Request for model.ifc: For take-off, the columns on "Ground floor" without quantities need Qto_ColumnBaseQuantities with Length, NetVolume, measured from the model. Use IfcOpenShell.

First a look at what the model holds.

```python
import ifcopenshell
import ifcopenshell.util.element
import ifcopenshell.util.unit

model = ifcopenshell.open("model.ifc")
print(model.schema)
for unit_type in ("LENGTHUNIT", "AREAUNIT", "VOLUMEUNIT"):
    print(unit_type, ifcopenshell.util.unit.calculate_unit_scale(model, unit_type))
storey = next(s for s in model.by_type("IfcBuildingStorey") if s.Name == "Ground floor")
columns = [e for e in ifcopenshell.util.element.get_decomposition(storey) if e.is_a("IfcColumn")]
for e in sorted(columns, key=lambda e: e.id()):
    print(e.id(), e.is_a(), e.Name, list(ifcopenshell.util.element.get_psets(e, qtos_only=True)), sep=" | ")
```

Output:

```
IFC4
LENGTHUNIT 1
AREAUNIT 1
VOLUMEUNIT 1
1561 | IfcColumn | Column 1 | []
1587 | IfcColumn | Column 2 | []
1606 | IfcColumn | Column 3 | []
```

```python
import ifcopenshell
import ifcopenshell.api.pset
import ifcopenshell.geom
import ifcopenshell.util.element
import ifcopenshell.util.shape
import ifcopenshell.util.unit

model = ifcopenshell.open("model.ifc")
unit_scale = ifcopenshell.util.unit.calculate_unit_scale(model)
volume_scale = ifcopenshell.util.unit.calculate_unit_scale(model, "VOLUMEUNIT")
settings = ifcopenshell.geom.settings()

storey = next(s for s in model.by_type("IfcBuildingStorey") if s.Name == "Ground floor")
columns = [e for e in ifcopenshell.util.element.get_decomposition(storey) if e.is_a("IfcColumn")]

for e in sorted(columns, key=lambda e: e.id()):
    if ifcopenshell.util.element.get_psets(e, qtos_only=True, should_inherit=False):
        continue
    # Geometry comes back in metres, in the element's own axes.
    shape = ifcopenshell.geom.create_shape(settings, e)
    values = {
        "Length": ifcopenshell.util.shape.get_z(shape.geometry) / unit_scale,
        "NetVolume": ifcopenshell.util.shape.get_volume(shape.geometry) / volume_scale,
    }
    qto = ifcopenshell.api.pset.add_qto(model, product=e, name="Qto_ColumnBaseQuantities")
    ifcopenshell.api.pset.edit_qto(model, qto=qto, properties=values)
    print(e.id(), {k: round(v, 3) for k, v in values.items()})

model.write("model_updated.ifc")
```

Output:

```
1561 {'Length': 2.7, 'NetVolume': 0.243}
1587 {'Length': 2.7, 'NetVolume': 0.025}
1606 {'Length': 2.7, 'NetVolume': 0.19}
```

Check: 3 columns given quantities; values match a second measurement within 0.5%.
